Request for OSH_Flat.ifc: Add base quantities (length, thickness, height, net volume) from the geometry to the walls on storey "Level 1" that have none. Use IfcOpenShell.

First a look at what the model holds.

```python
import ifcopenshell
import ifcopenshell.util.element
import ifcopenshell.util.unit

model = ifcopenshell.open("OSH_Flat.ifc")
print(model.schema)
for unit_type in ("LENGTHUNIT", "AREAUNIT", "VOLUMEUNIT"):
    print(unit_type, ifcopenshell.util.unit.calculate_unit_scale(model, unit_type))
storey = next(s for s in model.by_type("IfcBuildingStorey") if s.Name == "Level 1")
walls = [e for e in ifcopenshell.util.element.get_decomposition(storey) if e.is_a("IfcWall")]
for e in sorted(walls, key=lambda e: e.id()):
    print(e.id(), e.is_a(), e.Name, list(ifcopenshell.util.element.get_psets(e, qtos_only=True)), sep=" | ")
```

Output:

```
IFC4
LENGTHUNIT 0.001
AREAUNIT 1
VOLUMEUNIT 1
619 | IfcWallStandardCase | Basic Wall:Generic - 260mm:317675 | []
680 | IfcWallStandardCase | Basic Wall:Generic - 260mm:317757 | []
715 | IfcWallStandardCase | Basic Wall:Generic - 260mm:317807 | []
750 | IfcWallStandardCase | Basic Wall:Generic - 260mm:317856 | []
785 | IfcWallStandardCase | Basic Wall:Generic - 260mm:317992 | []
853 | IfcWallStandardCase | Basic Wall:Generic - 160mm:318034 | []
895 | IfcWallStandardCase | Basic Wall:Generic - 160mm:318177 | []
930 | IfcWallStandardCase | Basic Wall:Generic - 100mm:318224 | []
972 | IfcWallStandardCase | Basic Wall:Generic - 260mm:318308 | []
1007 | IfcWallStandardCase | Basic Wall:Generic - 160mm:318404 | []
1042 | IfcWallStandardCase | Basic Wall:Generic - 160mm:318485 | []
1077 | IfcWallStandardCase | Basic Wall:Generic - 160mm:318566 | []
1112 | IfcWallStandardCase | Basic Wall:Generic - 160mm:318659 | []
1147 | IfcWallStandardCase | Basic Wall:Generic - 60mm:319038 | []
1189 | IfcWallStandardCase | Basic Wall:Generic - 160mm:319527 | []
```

```python
import ifcopenshell
import ifcopenshell.api.pset
import ifcopenshell.geom
import ifcopenshell.util.element
import ifcopenshell.util.shape
import ifcopenshell.util.unit

model = ifcopenshell.open("OSH_Flat.ifc")
unit_scale = ifcopenshell.util.unit.calculate_unit_scale(model)
volume_scale = ifcopenshell.util.unit.calculate_unit_scale(model, "VOLUMEUNIT")
settings = ifcopenshell.geom.settings()

storey = next(s for s in model.by_type("IfcBuildingStorey") if s.Name == "Level 1")
walls = [e for e in ifcopenshell.util.element.get_decomposition(storey) if e.is_a("IfcWall")]

for e in sorted(walls, key=lambda e: e.id()):
    if ifcopenshell.util.element.get_psets(e, qtos_only=True, should_inherit=False):
        continue
    # Geometry comes back in metres, in the element's own axes.
    shape = ifcopenshell.geom.create_shape(settings, e)
    values = {
        "Length": ifcopenshell.util.shape.get_x(shape.geometry) / unit_scale,
        "Width": ifcopenshell.util.shape.get_y(shape.geometry) / unit_scale,
        "Height": ifcopenshell.util.shape.get_z(shape.geometry) / unit_scale,
        "NetVolume": ifcopenshell.util.shape.get_volume(shape.geometry) / volume_scale,
    }
    qto = ifcopenshell.api.pset.add_qto(model, product=e, name="Qto_WallBaseQuantities")
    ifcopenshell.api.pset.edit_qto(model, qto=qto, properties=values)
    print(e.id(), {k: round(v, 3) for k, v in values.items()})

model.write("OSH_Flat_edited.ifc")
```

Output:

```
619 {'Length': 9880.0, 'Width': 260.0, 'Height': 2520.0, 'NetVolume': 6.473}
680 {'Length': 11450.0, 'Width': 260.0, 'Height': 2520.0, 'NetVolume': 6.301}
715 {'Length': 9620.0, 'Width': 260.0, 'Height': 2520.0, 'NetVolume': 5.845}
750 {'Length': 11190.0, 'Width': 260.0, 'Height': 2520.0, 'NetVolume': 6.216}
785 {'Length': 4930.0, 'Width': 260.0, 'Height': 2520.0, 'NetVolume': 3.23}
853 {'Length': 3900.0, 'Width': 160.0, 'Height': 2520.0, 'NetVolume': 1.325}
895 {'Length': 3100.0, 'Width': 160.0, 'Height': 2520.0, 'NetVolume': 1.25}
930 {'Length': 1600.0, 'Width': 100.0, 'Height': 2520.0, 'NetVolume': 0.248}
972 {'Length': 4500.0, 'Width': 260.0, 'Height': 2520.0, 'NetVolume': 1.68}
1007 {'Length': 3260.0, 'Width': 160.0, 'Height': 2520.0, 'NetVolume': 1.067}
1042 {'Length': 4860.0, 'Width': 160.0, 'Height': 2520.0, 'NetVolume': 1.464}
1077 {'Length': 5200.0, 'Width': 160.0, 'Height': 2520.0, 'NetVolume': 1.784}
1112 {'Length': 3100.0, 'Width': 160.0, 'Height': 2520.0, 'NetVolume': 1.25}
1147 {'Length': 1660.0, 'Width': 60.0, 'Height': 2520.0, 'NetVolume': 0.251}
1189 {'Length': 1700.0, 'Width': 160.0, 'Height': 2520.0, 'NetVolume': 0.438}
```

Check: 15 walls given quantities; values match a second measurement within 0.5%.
